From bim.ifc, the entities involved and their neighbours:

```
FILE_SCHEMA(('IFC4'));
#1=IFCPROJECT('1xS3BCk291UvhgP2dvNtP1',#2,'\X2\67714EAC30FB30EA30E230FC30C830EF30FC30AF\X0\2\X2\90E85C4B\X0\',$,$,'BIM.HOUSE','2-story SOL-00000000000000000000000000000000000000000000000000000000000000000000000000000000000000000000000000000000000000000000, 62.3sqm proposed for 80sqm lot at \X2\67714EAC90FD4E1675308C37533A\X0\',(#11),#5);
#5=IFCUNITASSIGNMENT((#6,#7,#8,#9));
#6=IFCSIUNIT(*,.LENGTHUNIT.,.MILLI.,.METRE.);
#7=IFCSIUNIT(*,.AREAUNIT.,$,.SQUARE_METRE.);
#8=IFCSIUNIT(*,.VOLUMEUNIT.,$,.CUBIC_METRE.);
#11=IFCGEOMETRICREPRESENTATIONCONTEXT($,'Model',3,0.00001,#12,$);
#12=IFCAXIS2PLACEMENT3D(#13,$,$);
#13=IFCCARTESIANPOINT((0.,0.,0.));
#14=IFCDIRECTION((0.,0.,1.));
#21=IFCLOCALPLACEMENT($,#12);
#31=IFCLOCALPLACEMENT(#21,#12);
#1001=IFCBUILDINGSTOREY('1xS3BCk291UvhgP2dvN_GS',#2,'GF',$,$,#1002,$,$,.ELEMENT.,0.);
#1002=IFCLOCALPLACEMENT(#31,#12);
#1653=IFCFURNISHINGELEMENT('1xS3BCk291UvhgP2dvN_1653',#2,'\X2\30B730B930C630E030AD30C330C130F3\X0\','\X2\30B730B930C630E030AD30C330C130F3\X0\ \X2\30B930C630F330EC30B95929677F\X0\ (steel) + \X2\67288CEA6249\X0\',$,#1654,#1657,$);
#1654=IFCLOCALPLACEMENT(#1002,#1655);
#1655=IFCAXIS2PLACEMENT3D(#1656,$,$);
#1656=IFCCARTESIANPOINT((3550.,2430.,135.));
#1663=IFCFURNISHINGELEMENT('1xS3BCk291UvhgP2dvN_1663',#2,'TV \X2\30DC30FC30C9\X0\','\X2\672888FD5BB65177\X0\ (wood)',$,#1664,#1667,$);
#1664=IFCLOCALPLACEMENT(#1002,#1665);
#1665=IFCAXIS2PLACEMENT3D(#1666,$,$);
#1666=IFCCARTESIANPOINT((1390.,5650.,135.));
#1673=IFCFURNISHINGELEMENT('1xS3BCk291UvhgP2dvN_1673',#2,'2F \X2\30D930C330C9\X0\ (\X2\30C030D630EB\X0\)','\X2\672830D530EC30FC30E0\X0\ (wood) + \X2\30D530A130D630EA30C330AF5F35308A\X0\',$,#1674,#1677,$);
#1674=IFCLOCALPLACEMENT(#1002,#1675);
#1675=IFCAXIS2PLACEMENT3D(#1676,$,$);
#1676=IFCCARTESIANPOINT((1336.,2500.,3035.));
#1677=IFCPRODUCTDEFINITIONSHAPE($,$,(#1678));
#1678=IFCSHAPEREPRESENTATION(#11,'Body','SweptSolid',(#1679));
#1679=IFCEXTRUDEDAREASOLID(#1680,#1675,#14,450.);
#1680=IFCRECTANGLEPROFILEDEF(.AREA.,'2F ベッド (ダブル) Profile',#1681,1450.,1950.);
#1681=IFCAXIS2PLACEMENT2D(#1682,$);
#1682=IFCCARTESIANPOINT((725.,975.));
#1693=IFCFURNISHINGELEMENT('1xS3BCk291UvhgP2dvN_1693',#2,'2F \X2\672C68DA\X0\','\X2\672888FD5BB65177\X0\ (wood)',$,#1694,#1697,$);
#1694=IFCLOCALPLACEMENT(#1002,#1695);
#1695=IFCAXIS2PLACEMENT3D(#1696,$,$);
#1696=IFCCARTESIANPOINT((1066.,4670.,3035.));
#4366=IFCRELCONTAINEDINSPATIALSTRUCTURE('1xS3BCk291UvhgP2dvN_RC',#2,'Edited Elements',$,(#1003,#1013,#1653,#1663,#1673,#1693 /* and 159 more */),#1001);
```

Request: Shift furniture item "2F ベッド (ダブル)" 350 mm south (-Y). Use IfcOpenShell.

```python
import ifcopenshell
import ifcopenshell.api.geometry
import ifcopenshell.util.placement

model = ifcopenshell.open("bim.ifc")

item = model.by_guid("1xS3BCk291UvhgP2dvN_1673")
matrix = ifcopenshell.util.placement.get_local_placement(item.ObjectPlacement)
matrix[1, 3] -= 350.0
ifcopenshell.api.geometry.edit_object_placement(model, product=item, matrix=matrix, is_si=False)

print(ifcopenshell.util.placement.get_local_placement(item.ObjectPlacement).round(3) + 0.0)

model.write("bim_edited.ifc")
```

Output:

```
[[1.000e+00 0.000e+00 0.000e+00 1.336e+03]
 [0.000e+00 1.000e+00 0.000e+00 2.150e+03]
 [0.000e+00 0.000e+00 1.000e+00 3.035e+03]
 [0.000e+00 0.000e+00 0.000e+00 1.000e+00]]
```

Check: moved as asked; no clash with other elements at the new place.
